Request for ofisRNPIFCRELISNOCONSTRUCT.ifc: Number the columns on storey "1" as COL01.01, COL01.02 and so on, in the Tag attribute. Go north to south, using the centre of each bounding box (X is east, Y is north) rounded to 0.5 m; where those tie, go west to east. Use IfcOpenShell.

First a look at what the model holds.

```python
import ifcopenshell
import ifcopenshell.util.element
import ifcopenshell.util.placement

model = ifcopenshell.open("ofisRNPIFCRELISNOCONSTRUCT.ifc")
print(model.schema)
storey = next(s for s in model.by_type("IfcBuildingStorey") if s.Name == "1")
columns = [e for e in ifcopenshell.util.element.get_decomposition(storey) if e.is_a("IfcColumn")]
for e in sorted(columns, key=lambda e: e.id()):
    origin = ifcopenshell.util.placement.get_local_placement(e.ObjectPlacement)[:3, 3]
    print(e.id(), e.Tag, e.Name, origin.round(2) + 0.0, sep=" | ")
```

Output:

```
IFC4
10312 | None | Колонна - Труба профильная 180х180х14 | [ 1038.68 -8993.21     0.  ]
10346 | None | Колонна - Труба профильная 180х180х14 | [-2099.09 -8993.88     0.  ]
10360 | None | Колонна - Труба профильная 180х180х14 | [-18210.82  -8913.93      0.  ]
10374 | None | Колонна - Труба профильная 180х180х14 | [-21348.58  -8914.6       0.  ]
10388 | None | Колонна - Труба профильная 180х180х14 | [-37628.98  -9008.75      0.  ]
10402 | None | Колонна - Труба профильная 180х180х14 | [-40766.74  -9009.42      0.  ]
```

```python
import ifcopenshell
import ifcopenshell.geom
import ifcopenshell.util.element
import ifcopenshell.util.shape

model = ifcopenshell.open("ofisRNPIFCRELISNOCONSTRUCT.ifc")
settings = ifcopenshell.geom.settings()
settings.set("use-world-coords", True)


def centre(element):
    shape = ifcopenshell.geom.create_shape(settings, element)
    return ifcopenshell.util.shape.get_bbox_centroid(shape.geometry)


storey = next(s for s in model.by_type("IfcBuildingStorey") if s.Name == "1")
columns = [e for e in ifcopenshell.util.element.get_decomposition(storey) if e.is_a("IfcColumn")]

# Insertion points can sit at a corner or the storey origin, so sort by the geometry (in metres).
centres = {e: centre(e) for e in columns}
columns.sort(key=lambda e: (-round(centres[e][1] / 0.5), centres[e][0]))

for i, e in enumerate(columns, start=1):
    number = f"COL01.{i:02d}"
    e.Tag = number
    print(e.id(), number)

model.write("ofisRNPIFCRELISNOCONSTRUCT_updated.ifc")
```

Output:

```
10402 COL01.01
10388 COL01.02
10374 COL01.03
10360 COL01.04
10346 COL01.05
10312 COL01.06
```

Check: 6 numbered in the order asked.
